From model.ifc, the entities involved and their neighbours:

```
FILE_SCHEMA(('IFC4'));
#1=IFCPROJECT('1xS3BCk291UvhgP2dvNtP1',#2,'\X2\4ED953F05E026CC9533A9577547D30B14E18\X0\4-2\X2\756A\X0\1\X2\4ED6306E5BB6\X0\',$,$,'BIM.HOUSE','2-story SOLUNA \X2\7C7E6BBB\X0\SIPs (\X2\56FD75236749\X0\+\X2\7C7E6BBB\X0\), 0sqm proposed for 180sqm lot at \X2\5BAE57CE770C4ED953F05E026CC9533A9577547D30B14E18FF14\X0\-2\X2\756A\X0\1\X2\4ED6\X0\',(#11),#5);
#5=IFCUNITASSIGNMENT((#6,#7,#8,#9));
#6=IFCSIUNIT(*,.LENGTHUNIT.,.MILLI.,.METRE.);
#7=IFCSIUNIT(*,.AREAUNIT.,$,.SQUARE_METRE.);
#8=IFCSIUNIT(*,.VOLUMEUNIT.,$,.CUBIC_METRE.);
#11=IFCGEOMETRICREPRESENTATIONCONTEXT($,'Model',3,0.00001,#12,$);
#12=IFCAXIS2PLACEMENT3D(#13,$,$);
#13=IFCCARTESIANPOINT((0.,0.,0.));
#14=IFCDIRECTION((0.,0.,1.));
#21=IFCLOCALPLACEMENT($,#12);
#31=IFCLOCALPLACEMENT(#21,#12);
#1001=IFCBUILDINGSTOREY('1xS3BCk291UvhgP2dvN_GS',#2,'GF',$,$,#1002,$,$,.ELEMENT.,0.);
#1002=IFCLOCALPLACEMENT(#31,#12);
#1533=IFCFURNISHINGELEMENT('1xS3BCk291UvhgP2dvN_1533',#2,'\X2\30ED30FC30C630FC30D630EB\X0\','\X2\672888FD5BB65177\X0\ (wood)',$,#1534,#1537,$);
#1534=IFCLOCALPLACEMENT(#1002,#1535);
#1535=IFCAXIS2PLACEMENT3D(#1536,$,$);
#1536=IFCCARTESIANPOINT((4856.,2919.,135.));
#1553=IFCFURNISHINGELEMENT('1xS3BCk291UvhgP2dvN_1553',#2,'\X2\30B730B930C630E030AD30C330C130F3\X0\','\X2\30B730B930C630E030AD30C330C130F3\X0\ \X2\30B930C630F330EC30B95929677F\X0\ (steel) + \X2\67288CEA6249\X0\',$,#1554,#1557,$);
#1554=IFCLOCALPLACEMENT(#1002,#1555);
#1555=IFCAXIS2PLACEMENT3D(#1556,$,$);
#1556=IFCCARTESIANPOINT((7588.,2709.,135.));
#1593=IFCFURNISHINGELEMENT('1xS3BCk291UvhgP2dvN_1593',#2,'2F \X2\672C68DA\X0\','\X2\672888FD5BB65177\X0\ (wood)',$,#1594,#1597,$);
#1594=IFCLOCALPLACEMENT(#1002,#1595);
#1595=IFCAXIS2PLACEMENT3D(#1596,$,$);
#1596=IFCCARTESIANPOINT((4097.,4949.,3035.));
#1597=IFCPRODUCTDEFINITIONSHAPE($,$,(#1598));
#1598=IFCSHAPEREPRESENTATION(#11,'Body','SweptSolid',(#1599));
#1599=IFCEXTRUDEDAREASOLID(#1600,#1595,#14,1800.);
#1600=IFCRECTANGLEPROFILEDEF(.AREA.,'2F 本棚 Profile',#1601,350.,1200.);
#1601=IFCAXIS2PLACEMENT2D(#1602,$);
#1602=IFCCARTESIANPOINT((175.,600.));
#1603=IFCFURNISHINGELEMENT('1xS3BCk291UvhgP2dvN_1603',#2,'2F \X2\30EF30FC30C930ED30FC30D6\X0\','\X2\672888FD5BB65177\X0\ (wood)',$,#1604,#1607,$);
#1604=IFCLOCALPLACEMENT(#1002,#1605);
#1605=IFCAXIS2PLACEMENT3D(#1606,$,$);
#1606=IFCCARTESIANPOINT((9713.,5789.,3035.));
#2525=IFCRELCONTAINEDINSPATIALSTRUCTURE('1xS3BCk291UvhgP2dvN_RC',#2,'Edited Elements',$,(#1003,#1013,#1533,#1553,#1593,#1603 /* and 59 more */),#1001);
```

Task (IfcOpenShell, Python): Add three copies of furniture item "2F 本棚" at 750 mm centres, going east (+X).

```python
import numpy as np
import ifcopenshell
import ifcopenshell.api.geometry
import ifcopenshell.api.root
import ifcopenshell.util.element
import ifcopenshell.util.placement
import ifcopenshell.util.unit

model = ifcopenshell.open("model.ifc")
unit_scale = ifcopenshell.util.unit.calculate_unit_scale(model)


def reuse_history(source, copy):
    """copy_class also copies each property set's owner history, people and application; keep the originals."""
    for rel in copy.IsDefinedBy:
        if rel.is_a("IfcRelDefinesByProperties") and (history := rel.RelatingPropertyDefinition.OwnerHistory):
            rel.RelatingPropertyDefinition.OwnerHistory = source.OwnerHistory
            ifcopenshell.util.element.remove_deep2(model, history)


source = model.by_guid("1xS3BCk291UvhgP2dvN_1593")
base = ifcopenshell.util.placement.get_local_placement(source.ObjectPlacement)
step = np.array([1.0, 0.0, 0.0]) * 0.75 / unit_scale

for i in range(1, 4):
    copy = ifcopenshell.api.root.copy_class(model, product=source)
    copy.Representation = ifcopenshell.util.element.copy_deep(
        model, source.Representation, exclude=["IfcGeometricRepresentationContext", "IfcRepresentationMap"]
    )
    reuse_history(source, copy)
    matrix = base.copy()
    matrix[:3, 3] += i * step
    print("added at", matrix[:3, 3].round(3) + 0.0)
    ifcopenshell.api.geometry.edit_object_placement(model, product=copy, matrix=matrix, is_si=False)

model.write("model_edited.ifc")
```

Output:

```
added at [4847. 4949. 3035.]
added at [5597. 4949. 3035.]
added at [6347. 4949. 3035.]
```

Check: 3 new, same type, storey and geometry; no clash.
